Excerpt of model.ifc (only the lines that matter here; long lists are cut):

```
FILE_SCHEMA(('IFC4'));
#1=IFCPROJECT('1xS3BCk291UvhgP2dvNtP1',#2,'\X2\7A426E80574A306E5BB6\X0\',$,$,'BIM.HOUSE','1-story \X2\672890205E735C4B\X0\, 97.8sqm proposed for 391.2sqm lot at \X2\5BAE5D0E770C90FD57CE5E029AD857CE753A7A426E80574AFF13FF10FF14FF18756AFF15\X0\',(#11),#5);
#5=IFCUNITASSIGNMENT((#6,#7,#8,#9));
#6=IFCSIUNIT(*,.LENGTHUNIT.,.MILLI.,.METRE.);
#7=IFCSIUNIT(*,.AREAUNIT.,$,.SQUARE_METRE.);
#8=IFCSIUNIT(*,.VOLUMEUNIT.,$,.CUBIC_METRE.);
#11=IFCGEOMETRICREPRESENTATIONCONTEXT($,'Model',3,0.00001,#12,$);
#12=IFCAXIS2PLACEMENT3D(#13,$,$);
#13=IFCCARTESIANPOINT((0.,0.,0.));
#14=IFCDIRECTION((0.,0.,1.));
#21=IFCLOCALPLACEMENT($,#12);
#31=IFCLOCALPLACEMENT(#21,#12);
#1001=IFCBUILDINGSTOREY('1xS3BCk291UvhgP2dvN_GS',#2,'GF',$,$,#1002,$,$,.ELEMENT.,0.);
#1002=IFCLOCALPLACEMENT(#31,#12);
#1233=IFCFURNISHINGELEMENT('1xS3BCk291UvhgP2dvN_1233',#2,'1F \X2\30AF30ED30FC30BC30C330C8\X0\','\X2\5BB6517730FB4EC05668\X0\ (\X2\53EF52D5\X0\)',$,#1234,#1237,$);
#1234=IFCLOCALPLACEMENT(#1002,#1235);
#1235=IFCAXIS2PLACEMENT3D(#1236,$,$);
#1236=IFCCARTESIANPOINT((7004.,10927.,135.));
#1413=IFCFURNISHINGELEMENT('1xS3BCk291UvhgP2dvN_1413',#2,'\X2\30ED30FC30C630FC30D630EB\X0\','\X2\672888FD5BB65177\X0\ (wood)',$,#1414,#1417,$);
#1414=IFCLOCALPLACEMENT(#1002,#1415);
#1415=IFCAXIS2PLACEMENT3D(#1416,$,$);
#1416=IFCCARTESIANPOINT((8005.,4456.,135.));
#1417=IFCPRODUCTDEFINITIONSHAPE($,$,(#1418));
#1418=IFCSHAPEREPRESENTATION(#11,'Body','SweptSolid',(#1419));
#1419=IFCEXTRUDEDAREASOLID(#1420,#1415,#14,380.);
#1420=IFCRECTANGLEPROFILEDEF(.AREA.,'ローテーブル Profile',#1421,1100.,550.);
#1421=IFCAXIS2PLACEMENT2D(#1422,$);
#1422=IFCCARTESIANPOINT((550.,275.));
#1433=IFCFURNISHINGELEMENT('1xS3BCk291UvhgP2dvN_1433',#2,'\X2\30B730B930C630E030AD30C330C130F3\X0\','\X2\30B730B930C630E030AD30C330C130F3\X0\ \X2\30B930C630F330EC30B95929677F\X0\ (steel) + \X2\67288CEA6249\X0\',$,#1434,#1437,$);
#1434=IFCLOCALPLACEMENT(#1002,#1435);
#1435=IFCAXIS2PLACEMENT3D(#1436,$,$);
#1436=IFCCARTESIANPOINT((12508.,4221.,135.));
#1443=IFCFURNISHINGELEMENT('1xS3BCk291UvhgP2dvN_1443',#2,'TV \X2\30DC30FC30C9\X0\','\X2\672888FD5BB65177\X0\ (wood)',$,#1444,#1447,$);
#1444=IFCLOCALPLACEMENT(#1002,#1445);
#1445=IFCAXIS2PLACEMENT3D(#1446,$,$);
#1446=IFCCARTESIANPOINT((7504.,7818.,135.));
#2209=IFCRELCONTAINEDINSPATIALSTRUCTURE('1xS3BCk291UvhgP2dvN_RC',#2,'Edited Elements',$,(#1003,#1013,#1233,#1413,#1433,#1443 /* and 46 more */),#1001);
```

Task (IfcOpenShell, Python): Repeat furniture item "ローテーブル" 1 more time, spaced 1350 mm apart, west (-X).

```python
import numpy as np
import ifcopenshell
import ifcopenshell.api.geometry
import ifcopenshell.api.root
import ifcopenshell.util.element
import ifcopenshell.util.placement
import ifcopenshell.util.unit

model = ifcopenshell.open("model.ifc")
unit_scale = ifcopenshell.util.unit.calculate_unit_scale(model)


def reuse_history(source, copy):
    """copy_class also copies each property set's owner history, people and application; keep the originals."""
    for rel in copy.IsDefinedBy:
        if rel.is_a("IfcRelDefinesByProperties") and (history := rel.RelatingPropertyDefinition.OwnerHistory):
            rel.RelatingPropertyDefinition.OwnerHistory = source.OwnerHistory
            ifcopenshell.util.element.remove_deep2(model, history)


source = model.by_guid("1xS3BCk291UvhgP2dvN_1413")
base = ifcopenshell.util.placement.get_local_placement(source.ObjectPlacement)
step = np.array([-1.0, 0.0, 0.0]) * 1.35 / unit_scale

for i in range(1, 2):
    copy = ifcopenshell.api.root.copy_class(model, product=source)
    copy.Representation = ifcopenshell.util.element.copy_deep(
        model, source.Representation, exclude=["IfcGeometricRepresentationContext", "IfcRepresentationMap"]
    )
    reuse_history(source, copy)
    matrix = base.copy()
    matrix[:3, 3] += i * step
    print("added at", matrix[:3, 3].round(3) + 0.0)
    ifcopenshell.api.geometry.edit_object_placement(model, product=copy, matrix=matrix, is_si=False)

model.write("model_rev.ifc")
```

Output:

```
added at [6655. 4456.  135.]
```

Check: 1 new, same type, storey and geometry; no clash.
